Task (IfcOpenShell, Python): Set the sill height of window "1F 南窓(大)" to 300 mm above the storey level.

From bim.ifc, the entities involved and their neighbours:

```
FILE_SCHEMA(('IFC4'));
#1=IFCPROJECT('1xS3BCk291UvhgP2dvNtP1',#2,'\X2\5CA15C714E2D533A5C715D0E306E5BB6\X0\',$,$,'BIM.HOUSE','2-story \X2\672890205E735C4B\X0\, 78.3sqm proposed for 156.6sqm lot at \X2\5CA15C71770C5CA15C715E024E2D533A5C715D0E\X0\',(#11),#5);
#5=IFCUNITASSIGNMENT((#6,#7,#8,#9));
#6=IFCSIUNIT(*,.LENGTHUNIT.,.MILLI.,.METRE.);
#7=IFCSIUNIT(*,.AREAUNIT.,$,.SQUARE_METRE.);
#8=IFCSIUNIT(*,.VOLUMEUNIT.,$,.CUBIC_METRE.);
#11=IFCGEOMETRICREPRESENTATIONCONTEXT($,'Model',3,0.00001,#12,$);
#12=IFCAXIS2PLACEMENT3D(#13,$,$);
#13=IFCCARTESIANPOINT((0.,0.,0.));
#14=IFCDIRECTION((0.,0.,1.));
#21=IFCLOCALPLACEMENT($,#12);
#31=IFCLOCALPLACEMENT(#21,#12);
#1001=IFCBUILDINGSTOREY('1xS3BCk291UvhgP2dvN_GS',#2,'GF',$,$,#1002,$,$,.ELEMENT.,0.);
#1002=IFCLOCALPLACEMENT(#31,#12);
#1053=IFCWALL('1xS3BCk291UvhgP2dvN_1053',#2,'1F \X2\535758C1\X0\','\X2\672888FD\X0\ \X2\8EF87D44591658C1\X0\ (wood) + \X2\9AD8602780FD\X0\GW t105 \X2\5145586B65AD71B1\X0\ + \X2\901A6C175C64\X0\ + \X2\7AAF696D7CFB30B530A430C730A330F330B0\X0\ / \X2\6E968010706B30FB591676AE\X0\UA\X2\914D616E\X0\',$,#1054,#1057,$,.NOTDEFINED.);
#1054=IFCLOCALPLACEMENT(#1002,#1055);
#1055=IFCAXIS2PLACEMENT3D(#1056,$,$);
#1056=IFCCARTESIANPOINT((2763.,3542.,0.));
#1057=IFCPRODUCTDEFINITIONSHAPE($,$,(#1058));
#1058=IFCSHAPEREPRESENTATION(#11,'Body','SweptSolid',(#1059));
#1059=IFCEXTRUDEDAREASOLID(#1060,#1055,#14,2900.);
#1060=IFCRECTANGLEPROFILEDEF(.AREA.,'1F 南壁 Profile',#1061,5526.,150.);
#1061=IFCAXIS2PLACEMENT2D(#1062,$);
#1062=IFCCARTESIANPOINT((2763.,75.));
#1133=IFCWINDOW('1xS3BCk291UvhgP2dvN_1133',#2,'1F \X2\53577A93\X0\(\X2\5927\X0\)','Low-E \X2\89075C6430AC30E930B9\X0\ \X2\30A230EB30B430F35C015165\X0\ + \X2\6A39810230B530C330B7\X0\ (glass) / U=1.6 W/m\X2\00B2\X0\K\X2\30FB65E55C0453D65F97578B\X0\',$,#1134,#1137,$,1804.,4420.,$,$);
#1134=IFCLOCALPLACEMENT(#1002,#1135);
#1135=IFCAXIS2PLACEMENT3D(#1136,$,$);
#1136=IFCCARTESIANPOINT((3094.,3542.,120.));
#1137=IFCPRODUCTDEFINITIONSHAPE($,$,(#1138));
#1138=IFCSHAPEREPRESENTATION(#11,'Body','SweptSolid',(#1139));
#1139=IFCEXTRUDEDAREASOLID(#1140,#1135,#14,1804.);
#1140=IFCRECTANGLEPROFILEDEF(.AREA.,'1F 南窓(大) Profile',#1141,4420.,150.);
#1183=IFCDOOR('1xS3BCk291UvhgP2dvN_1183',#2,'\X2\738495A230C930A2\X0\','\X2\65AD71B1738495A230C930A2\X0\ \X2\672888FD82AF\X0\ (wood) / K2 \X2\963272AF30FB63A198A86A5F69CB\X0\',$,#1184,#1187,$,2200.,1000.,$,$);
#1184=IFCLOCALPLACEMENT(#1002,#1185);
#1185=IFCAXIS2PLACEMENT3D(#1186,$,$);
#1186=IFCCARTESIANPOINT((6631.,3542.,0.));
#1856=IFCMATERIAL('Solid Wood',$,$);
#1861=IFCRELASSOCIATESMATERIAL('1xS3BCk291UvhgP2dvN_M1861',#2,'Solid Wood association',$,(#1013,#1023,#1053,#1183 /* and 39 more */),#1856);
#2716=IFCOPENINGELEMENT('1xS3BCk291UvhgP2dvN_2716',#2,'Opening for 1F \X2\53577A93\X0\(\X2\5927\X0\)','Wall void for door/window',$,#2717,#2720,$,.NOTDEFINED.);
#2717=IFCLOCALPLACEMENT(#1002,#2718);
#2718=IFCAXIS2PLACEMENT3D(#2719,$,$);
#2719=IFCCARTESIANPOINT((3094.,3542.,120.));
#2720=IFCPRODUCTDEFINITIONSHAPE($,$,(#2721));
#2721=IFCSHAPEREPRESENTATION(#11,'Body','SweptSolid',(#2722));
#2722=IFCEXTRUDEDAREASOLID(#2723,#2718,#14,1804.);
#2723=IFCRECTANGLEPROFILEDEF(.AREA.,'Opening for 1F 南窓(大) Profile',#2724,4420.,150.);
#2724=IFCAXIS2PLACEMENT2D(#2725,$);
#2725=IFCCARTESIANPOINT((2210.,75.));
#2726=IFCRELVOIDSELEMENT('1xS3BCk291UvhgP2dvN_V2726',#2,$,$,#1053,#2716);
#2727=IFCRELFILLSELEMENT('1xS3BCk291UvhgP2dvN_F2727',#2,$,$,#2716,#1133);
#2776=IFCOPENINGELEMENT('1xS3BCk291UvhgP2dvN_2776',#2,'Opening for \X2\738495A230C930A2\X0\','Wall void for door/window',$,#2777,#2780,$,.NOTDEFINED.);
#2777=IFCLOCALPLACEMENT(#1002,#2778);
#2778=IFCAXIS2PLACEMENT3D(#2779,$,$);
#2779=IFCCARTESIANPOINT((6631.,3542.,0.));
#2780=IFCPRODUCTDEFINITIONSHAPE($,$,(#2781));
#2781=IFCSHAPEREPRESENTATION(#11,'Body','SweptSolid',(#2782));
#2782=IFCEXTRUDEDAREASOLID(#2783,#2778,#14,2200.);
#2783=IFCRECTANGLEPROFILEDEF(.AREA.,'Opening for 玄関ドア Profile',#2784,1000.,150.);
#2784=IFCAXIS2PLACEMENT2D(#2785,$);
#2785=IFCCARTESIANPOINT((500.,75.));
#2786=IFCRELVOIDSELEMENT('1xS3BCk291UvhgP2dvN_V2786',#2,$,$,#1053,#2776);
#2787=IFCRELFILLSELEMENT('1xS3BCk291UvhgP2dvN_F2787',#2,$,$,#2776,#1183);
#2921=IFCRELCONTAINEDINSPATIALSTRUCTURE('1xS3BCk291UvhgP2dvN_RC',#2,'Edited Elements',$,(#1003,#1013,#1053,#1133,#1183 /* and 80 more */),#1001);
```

```python
import numpy as np
import ifcopenshell
import ifcopenshell.api.geometry
import ifcopenshell.geom
import ifcopenshell.util.element
import ifcopenshell.util.placement
import ifcopenshell.util.shape
import ifcopenshell.util.unit

model = ifcopenshell.open("bim.ifc")
unit_scale = ifcopenshell.util.unit.calculate_unit_scale(model)

window = model.by_guid("1xS3BCk291UvhgP2dvN_1133")
opening = window.FillsVoids[0].RelatingOpeningElement
storey = ifcopenshell.util.element.get_container(window, ifc_class="IfcBuildingStorey")
level = ifcopenshell.util.placement.get_local_placement(storey.ObjectPlacement)[2, 3]

# The opening's origin need not be at the sill, so measure its lowest point.
shape = ifcopenshell.geom.create_shape(ifcopenshell.geom.settings(), opening)
bottom = ifcopenshell.util.shape.get_shape_bottom_elevation(shape, shape.geometry) / unit_scale
dz = level + 300.0 - bottom

shift = np.array([0.0, 0.0, dz])
# The window is not placed relative to its opening, so move both.
for product in (opening, window):
    matrix = ifcopenshell.util.placement.get_local_placement(product.ObjectPlacement)
    matrix[:3, 3] += shift
    ifcopenshell.api.geometry.edit_object_placement(model, product=product, matrix=matrix, is_si=False)

print(f"moved by {dz * unit_scale:+.3f} m")

model.write("bim_updated.ifc")
```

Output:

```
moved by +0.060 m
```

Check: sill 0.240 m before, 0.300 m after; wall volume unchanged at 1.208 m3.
